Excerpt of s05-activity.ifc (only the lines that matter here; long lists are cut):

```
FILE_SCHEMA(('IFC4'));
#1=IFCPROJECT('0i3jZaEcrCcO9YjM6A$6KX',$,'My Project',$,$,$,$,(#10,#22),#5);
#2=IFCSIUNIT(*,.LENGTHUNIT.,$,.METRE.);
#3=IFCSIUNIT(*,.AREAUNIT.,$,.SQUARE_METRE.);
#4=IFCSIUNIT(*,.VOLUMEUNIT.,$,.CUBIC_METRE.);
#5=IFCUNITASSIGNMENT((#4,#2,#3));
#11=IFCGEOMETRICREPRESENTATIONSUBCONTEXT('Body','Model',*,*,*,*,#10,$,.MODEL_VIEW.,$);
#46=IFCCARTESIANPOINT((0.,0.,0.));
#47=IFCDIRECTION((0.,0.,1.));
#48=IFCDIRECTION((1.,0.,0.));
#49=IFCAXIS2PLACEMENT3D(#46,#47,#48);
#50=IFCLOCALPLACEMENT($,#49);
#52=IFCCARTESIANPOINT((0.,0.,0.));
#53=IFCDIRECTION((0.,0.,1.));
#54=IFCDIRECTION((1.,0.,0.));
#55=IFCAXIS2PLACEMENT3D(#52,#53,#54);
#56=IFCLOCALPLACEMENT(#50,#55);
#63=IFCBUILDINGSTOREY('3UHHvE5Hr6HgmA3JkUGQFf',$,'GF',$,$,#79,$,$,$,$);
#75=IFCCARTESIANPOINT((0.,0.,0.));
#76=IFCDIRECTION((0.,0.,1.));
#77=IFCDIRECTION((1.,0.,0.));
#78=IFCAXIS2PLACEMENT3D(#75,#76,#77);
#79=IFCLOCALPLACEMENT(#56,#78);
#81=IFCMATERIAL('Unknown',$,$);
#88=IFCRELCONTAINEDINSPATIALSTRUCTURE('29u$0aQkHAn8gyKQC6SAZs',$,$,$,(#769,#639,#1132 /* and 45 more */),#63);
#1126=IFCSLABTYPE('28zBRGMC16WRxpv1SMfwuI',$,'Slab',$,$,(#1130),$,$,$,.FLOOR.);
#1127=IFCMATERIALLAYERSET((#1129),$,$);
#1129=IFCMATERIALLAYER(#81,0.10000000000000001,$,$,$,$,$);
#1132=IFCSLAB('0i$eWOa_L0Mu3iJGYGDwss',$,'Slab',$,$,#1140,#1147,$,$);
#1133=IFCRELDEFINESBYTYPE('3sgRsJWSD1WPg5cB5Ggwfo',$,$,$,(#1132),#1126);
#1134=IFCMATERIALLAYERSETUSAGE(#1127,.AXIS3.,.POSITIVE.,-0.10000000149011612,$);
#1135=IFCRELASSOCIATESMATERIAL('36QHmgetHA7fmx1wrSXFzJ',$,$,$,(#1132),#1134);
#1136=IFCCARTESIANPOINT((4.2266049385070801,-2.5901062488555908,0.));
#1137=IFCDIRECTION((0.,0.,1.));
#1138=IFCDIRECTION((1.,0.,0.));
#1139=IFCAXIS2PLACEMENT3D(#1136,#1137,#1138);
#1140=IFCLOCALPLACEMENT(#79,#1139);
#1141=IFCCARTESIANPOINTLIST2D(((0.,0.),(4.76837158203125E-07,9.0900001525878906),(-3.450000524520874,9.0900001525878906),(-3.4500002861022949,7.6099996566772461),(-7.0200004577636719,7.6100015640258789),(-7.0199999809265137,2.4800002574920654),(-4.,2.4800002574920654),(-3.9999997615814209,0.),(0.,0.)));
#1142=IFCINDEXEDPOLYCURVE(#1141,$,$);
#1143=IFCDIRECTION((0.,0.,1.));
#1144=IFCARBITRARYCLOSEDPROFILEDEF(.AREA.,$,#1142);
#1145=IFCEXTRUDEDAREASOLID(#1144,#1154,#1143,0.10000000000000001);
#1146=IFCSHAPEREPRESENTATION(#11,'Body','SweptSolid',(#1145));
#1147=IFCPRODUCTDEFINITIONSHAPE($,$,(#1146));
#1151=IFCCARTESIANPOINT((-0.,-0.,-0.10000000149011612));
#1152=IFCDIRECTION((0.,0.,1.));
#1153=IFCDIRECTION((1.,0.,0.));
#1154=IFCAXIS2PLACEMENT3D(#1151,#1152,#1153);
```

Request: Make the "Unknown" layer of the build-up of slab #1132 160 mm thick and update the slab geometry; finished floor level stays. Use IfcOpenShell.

```python
import ifcopenshell
import ifcopenshell.util.element
import ifcopenshell.util.representation

model = ifcopenshell.open("s05-activity.ifc")

layer_set = model.by_id(1127)
layer = next(l for l in layer_set.MaterialLayers if l.Material and l.Material.Name == "Unknown")
change = 0.16 - layer.LayerThickness
layer.LayerThickness += change

# Geometry does not follow the layer set by itself.
slabs = [e for e in ifcopenshell.util.element.get_elements_by_material(model, layer_set) if e.is_a("IfcSlab")]
for slab in sorted(slabs, key=lambda e: e.id()):
    body = ifcopenshell.util.representation.get_representation(slab, "Model", "Body")
    solid = body.Items[0]
    old_depth = solid.Depth
    solid.Depth += change
    # Extruded upwards: lower the start of the extrusion so the top stays.
    x, y, z = solid.Position.Location.Coordinates
    solid.Position.Location = model.createIfcCartesianPoint((x, y, z - change))
    print(slab.id(), f"{old_depth:g} -> {solid.Depth:g}")

# The layers are counted up from the underside, which has moved.
for usage in {ifcopenshell.util.element.get_material(slab) for slab in slabs}:
    usage.OffsetFromReferenceLine -= change

model.write("s05-activity_v2.ifc")
```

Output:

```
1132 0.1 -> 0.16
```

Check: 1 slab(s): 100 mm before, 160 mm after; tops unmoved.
